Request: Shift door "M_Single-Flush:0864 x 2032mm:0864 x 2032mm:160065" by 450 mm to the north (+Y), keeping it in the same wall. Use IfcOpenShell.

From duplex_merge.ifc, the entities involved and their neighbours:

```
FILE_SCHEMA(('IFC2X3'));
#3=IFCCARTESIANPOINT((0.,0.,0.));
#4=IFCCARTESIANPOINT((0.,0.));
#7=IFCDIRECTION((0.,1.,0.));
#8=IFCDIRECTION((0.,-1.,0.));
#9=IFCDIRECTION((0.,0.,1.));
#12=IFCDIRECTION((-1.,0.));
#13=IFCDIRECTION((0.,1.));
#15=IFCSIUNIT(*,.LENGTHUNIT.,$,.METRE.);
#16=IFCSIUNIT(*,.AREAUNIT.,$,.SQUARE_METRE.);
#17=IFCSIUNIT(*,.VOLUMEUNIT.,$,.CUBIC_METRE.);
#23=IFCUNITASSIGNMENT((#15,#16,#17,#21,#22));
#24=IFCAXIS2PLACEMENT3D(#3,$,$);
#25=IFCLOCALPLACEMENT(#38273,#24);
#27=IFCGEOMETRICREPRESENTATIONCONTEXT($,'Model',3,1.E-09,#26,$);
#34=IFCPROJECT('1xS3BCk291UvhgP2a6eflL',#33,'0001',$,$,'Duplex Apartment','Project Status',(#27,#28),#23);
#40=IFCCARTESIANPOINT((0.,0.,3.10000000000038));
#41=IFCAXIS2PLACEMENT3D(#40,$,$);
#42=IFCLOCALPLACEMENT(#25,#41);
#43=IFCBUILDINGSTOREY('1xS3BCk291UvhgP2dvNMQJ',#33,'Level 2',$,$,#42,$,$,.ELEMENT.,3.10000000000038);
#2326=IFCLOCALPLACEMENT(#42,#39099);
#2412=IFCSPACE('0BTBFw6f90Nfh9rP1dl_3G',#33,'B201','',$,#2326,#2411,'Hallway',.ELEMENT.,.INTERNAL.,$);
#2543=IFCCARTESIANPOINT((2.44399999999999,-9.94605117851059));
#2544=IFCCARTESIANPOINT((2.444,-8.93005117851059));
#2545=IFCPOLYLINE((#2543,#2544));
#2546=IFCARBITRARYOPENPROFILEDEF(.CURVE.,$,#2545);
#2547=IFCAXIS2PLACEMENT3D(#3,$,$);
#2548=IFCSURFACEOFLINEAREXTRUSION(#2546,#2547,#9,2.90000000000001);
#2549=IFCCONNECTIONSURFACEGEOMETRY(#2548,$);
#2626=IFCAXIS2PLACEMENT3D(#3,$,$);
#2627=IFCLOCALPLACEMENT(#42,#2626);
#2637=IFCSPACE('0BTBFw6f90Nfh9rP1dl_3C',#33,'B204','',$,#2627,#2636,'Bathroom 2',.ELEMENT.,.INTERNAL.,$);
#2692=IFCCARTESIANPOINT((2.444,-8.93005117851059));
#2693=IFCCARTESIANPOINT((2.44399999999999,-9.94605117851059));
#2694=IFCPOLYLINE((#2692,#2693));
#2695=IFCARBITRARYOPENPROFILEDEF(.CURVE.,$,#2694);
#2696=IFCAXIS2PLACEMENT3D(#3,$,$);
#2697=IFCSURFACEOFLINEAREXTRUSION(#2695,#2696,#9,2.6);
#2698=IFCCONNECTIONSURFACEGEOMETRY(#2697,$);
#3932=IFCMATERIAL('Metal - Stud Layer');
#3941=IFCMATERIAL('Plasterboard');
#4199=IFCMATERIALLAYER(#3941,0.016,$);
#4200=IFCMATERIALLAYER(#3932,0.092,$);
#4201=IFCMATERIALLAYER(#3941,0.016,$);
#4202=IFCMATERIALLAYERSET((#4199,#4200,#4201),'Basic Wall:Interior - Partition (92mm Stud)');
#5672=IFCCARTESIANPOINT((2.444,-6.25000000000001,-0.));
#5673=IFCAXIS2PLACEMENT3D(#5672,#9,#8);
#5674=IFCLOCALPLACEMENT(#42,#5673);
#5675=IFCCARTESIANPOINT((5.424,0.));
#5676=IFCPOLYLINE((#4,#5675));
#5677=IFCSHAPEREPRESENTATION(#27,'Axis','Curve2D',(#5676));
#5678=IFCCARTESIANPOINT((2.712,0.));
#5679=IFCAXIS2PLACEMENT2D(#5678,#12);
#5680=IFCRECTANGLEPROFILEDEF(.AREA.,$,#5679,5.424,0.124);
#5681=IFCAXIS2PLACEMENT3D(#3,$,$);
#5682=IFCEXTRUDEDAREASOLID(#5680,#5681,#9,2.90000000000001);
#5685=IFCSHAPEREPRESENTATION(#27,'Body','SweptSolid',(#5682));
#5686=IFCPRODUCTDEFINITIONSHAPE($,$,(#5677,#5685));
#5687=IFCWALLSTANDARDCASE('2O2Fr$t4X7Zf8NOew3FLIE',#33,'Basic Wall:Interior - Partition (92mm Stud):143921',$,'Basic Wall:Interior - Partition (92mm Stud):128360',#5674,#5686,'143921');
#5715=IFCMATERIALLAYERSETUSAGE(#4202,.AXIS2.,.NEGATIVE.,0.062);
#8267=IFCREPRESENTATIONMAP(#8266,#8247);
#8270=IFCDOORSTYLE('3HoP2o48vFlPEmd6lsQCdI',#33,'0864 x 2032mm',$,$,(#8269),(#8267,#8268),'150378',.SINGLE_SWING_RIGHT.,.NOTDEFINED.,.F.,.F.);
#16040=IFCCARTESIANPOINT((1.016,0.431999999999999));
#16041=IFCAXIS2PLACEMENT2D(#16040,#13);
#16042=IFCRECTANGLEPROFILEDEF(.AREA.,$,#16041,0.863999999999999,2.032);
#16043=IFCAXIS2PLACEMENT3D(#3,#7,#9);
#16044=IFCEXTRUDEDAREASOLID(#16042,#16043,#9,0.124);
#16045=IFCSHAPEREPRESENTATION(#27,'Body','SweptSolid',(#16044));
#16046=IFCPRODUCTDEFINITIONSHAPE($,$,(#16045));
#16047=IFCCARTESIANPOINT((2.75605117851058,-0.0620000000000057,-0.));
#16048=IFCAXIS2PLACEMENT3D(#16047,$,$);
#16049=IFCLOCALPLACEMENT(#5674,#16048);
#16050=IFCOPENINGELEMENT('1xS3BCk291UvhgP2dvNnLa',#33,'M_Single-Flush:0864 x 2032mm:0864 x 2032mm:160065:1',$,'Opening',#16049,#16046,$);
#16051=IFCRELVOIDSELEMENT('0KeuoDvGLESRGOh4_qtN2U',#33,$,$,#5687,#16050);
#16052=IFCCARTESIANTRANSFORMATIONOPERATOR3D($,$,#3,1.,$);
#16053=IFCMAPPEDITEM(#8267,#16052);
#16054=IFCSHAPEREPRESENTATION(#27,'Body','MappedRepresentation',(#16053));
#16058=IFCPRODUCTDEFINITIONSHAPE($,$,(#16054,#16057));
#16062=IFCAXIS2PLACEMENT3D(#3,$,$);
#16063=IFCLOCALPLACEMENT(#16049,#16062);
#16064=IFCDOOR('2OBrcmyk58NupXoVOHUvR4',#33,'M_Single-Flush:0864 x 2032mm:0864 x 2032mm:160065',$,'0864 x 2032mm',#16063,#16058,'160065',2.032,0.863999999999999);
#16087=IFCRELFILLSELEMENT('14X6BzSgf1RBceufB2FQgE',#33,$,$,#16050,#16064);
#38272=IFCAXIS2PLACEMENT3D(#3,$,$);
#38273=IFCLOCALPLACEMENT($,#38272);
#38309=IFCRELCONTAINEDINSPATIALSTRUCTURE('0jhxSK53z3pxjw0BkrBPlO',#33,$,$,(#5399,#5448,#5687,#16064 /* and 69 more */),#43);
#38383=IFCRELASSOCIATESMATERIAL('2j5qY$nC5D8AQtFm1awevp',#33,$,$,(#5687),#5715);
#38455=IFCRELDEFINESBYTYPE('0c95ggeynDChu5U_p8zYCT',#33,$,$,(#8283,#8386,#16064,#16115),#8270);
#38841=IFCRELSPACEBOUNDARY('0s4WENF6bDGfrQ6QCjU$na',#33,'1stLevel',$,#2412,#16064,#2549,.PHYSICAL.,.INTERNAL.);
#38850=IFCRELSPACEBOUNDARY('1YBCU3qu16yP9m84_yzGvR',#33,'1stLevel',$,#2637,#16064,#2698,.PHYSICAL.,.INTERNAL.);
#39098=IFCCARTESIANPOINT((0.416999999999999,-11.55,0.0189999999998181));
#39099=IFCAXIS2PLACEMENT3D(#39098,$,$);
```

```python
import numpy as np
import ifcopenshell
import ifcopenshell.api.geometry
import ifcopenshell.util.placement

model = ifcopenshell.open("duplex_merge.ifc")

door = model.by_guid("2OBrcmyk58NupXoVOHUvR4")
opening = door.FillsVoids[0].RelatingOpeningElement
wall = opening.VoidsElements[0].RelatingBuildingElement

wall_matrix = ifcopenshell.util.placement.get_local_placement(wall.ObjectPlacement)
shift = wall_matrix[:3, 0] * -0.45
before = ifcopenshell.util.placement.get_local_placement(door.ObjectPlacement)[:3, 3].copy()

# The door is placed relative to its opening, so it follows when the opening moves.
matrix = ifcopenshell.util.placement.get_local_placement(opening.ObjectPlacement)
matrix[:3, 3] += shift
ifcopenshell.api.geometry.edit_object_placement(
    model, product=opening, matrix=matrix, is_si=False, should_transform_children=True
)

# Space boundary surfaces are stored in each space's coordinates; move them too.
for rel in door.ProvidesBoundaries:
    if not rel.ConnectionGeometry:
        continue
    surface = rel.ConnectionGeometry.SurfaceOnRelatingElement
    space_matrix = ifcopenshell.util.placement.get_local_placement(rel.RelatingSpace.ObjectPlacement)
    point = np.array(surface.Position.Location.Coordinates) + space_matrix[:3, :3].T @ shift
    surface.Position = model.createIfcAxis2Placement3D(
        model.createIfcCartesianPoint(point.tolist()), surface.Position.Axis, surface.Position.RefDirection
    )

after = ifcopenshell.util.placement.get_local_placement(door.ObjectPlacement)[:3, 3]
print("door moved by", (after - before).round(3) + 0.0)

model.write("duplex_merge_edited.ifc")
```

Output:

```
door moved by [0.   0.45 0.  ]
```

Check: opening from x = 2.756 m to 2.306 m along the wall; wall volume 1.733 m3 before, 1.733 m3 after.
